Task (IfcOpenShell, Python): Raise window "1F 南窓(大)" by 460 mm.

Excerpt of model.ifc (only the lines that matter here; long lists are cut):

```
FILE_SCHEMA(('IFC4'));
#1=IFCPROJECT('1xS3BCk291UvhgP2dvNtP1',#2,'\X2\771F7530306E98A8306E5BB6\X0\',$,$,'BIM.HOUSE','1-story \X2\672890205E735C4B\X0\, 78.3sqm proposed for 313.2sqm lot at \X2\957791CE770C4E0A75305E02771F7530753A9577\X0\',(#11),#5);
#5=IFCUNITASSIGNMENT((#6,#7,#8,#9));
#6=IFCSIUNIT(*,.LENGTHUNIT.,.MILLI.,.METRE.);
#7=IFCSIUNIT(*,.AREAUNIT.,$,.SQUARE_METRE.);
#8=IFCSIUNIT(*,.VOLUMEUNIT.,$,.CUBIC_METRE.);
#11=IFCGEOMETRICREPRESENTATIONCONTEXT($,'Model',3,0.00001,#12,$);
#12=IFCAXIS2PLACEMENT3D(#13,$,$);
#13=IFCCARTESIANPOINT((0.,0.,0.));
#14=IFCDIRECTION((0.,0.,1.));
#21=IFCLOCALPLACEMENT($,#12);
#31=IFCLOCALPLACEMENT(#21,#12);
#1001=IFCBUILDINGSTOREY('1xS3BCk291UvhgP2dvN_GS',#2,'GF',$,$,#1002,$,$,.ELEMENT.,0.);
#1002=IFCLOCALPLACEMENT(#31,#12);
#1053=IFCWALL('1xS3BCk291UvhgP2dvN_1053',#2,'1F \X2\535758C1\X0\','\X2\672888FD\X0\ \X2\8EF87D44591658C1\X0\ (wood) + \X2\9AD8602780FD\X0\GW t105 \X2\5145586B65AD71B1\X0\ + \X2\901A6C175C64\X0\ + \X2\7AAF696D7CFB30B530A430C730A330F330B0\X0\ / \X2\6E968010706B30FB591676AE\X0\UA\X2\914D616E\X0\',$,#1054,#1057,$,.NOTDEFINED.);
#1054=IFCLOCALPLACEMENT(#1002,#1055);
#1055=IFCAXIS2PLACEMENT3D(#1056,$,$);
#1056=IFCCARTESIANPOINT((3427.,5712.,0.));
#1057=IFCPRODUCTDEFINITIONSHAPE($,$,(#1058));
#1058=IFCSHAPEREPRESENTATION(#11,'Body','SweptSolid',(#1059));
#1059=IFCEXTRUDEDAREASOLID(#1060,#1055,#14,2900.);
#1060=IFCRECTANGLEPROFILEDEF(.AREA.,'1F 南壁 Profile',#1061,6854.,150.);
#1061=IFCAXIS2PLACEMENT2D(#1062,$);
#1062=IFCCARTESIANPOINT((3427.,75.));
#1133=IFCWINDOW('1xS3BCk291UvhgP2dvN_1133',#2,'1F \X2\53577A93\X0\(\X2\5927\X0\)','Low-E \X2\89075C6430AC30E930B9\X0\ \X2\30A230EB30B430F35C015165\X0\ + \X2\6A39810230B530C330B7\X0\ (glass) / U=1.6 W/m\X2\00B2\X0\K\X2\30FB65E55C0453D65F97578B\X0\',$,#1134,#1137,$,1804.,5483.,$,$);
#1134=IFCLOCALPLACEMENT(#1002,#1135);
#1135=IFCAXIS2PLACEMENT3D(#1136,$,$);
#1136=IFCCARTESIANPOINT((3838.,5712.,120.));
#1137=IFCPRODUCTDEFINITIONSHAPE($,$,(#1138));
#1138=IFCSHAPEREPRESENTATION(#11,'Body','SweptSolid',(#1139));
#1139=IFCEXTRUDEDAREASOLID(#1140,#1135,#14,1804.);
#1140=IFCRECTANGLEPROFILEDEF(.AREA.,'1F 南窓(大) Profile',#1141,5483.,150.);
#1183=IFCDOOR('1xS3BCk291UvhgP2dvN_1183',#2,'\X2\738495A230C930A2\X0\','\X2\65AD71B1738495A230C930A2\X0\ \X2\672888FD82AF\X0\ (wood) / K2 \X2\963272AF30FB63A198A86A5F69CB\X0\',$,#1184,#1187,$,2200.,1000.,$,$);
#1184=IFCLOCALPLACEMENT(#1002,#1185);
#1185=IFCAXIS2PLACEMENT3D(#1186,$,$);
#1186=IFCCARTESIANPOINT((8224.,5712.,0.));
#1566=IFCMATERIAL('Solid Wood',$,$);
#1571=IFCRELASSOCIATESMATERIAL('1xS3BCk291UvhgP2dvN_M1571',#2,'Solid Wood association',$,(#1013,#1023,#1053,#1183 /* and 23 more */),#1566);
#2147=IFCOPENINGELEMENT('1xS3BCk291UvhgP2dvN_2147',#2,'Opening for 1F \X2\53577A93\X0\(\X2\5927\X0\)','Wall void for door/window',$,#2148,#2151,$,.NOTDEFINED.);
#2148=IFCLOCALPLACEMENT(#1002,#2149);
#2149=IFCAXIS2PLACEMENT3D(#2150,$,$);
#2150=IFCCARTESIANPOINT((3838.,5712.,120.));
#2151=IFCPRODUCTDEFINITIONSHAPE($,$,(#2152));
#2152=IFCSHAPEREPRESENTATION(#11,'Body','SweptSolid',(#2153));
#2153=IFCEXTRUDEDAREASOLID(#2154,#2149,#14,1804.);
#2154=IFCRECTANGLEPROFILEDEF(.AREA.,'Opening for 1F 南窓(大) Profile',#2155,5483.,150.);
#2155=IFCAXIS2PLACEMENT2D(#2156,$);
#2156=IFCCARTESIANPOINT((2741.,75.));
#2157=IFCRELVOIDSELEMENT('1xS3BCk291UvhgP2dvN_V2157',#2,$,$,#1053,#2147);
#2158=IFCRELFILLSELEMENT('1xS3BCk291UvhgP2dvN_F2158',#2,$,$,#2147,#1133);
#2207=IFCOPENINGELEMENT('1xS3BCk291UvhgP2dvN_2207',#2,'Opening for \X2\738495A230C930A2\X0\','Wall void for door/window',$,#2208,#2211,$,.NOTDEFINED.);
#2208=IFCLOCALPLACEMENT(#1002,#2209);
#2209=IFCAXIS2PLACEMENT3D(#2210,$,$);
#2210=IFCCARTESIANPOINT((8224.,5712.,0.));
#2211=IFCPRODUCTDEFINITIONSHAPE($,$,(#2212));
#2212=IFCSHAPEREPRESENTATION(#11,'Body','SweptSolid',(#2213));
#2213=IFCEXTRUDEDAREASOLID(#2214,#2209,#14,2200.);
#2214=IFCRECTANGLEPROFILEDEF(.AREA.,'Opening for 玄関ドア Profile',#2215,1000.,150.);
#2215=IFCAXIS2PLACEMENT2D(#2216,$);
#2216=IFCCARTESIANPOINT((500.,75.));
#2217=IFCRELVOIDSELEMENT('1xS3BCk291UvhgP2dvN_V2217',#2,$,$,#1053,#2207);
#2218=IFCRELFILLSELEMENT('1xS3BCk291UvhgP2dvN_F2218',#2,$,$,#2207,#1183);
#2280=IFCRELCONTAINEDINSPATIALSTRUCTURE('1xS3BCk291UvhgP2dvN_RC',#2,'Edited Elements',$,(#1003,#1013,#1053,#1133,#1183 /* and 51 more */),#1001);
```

```python
import numpy as np
import ifcopenshell
import ifcopenshell.api.geometry
import ifcopenshell.util.placement
import ifcopenshell.util.unit

model = ifcopenshell.open("model.ifc")
unit_scale = ifcopenshell.util.unit.calculate_unit_scale(model)

window = model.by_id(1133)
opening = window.FillsVoids[0].RelatingOpeningElement
dz = 460.0

shift = np.array([0.0, 0.0, dz])
# The window is not placed relative to its opening, so move both.
for product in (opening, window):
    matrix = ifcopenshell.util.placement.get_local_placement(product.ObjectPlacement)
    matrix[:3, 3] += shift
    ifcopenshell.api.geometry.edit_object_placement(model, product=product, matrix=matrix, is_si=False)

print(f"moved by {dz * unit_scale:+.3f} m")

model.write("model_rev.ifc")
```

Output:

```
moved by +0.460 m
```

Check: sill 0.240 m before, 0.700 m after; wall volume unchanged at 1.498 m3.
